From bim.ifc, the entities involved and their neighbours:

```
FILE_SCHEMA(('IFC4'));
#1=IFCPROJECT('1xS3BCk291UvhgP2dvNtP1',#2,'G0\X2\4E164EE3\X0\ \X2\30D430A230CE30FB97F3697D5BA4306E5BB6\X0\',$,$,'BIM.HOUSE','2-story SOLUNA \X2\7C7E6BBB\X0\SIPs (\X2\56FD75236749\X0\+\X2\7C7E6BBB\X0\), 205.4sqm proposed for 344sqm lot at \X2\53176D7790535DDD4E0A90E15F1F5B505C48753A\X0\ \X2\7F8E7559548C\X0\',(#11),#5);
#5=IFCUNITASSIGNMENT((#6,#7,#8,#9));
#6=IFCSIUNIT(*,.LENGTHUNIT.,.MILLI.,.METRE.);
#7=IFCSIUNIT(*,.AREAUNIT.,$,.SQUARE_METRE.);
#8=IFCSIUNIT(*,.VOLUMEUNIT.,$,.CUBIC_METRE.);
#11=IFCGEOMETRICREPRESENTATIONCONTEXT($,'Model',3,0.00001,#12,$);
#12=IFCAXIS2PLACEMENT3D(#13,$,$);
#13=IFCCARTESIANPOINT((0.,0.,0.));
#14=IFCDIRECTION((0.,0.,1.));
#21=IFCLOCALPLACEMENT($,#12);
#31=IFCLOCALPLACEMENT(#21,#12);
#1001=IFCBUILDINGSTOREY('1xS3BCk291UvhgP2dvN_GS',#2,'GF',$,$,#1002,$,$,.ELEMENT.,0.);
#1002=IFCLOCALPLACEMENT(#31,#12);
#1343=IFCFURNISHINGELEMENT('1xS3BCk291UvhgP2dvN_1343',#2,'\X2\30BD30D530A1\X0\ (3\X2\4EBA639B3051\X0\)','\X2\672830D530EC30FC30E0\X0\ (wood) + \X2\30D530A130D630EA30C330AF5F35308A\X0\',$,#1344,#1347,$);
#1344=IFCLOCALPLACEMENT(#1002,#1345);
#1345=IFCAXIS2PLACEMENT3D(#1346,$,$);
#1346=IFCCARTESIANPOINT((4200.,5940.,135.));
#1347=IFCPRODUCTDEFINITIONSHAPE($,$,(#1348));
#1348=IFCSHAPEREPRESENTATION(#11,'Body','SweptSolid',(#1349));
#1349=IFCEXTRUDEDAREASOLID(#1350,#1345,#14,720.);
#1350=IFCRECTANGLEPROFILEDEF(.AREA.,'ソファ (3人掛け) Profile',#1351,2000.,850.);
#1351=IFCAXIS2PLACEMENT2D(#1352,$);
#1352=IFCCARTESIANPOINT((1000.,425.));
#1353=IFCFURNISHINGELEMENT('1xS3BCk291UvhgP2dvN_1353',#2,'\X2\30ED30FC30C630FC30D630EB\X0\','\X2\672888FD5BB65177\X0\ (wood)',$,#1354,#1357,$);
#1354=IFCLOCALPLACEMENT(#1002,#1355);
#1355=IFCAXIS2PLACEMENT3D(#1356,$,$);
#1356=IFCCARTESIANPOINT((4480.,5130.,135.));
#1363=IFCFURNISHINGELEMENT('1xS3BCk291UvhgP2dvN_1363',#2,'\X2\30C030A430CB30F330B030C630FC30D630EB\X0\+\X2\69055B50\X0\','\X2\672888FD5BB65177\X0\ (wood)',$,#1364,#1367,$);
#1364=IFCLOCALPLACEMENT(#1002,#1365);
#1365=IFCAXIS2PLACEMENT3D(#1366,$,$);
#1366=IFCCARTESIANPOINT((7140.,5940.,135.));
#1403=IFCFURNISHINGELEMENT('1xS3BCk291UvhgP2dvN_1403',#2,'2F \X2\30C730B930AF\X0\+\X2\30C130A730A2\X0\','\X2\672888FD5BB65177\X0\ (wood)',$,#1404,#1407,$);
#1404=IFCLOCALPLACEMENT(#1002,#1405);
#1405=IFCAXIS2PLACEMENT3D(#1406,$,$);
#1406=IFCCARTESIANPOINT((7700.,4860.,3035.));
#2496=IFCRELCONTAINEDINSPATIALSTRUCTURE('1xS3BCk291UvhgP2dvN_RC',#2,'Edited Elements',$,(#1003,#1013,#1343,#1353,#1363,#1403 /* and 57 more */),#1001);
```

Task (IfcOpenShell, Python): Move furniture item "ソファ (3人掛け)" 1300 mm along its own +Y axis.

```python
import ifcopenshell
import ifcopenshell.api.geometry
import ifcopenshell.util.placement

model = ifcopenshell.open("bim.ifc")

item = model.by_guid("1xS3BCk291UvhgP2dvN_1343")
matrix = ifcopenshell.util.placement.get_local_placement(item.ObjectPlacement)
matrix[:3, 3] += matrix[:3, 1] * 1300.0
ifcopenshell.api.geometry.edit_object_placement(model, product=item, matrix=matrix, is_si=False)

print(ifcopenshell.util.placement.get_local_placement(item.ObjectPlacement).round(3) + 0.0)

model.write("bim_updated.ifc")
```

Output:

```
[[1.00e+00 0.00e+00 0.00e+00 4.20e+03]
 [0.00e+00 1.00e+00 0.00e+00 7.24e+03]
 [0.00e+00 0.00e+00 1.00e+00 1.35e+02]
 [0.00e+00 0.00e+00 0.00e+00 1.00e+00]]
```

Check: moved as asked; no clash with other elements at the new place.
